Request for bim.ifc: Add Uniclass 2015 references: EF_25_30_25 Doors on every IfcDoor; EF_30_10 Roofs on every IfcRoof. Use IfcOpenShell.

First a look at what the model holds.

```python
import ifcopenshell

model = ifcopenshell.open("bim.ifc")
print(model.schema)
print("classifications:", [c.Name for c in model.by_type("IfcClassification")])
for ifc_class in ("IfcDoor", "IfcRoof", "IfcStair", "IfcWall", "IfcWindow"):
    print(ifc_class, len(model.by_type(ifc_class)))
```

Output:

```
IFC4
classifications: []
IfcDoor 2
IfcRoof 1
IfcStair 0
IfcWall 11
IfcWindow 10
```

```python
import ifcopenshell
import ifcopenshell.api.classification

model = ifcopenshell.open("bim.ifc")

system = ifcopenshell.api.classification.add_classification(model, classification="Uniclass 2015")

codes = {
    "IfcDoor": ("EF_25_30_25", "Doors"),
    "IfcRoof": ("EF_30_10", "Roofs"),
}
for ifc_class, (code, name) in codes.items():
    products = model.by_type(ifc_class)
    ifcopenshell.api.classification.add_reference(
        model, products=products, classification=system, identification=code, name=name
    )
    print(code, len(products))

model.write("bim_updated.ifc")
```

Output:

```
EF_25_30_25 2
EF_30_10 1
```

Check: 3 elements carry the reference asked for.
